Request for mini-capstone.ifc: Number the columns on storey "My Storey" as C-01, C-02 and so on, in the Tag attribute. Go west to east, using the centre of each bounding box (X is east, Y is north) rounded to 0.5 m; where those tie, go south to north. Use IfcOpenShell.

First a look at what the model holds.

```python
import ifcopenshell
import ifcopenshell.util.element
import ifcopenshell.util.placement

model = ifcopenshell.open("mini-capstone.ifc")
print(model.schema)
storey = next(s for s in model.by_type("IfcBuildingStorey") if s.Name == "My Storey")
columns = [e for e in ifcopenshell.util.element.get_decomposition(storey) if e.is_a("IfcColumn")]
for e in sorted(columns, key=lambda e: e.id()):
    origin = ifcopenshell.util.placement.get_local_placement(e.ObjectPlacement)[:3, 3]
    print(e.id(), e.Tag, e.Name, origin.round(2) + 0.0, sep=" | ")
```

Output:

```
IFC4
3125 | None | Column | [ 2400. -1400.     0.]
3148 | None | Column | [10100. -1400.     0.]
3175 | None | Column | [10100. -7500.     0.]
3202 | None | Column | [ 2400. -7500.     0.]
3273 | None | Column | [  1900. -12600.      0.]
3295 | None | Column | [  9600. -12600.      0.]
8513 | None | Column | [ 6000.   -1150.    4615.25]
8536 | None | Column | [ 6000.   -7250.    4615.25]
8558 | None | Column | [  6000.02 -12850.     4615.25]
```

```python
import ifcopenshell
import ifcopenshell.geom
import ifcopenshell.util.element
import ifcopenshell.util.shape

model = ifcopenshell.open("mini-capstone.ifc")
settings = ifcopenshell.geom.settings()
settings.set("use-world-coords", True)


def centre(element):
    shape = ifcopenshell.geom.create_shape(settings, element)
    return ifcopenshell.util.shape.get_bbox_centroid(shape.geometry)


storey = next(s for s in model.by_type("IfcBuildingStorey") if s.Name == "My Storey")
columns = [e for e in ifcopenshell.util.element.get_decomposition(storey) if e.is_a("IfcColumn")]

# Insertion points can sit at a corner or the storey origin, so sort by the geometry (in metres).
centres = {e: centre(e) for e in columns}
columns.sort(key=lambda e: (round(centres[e][0] / 0.5), centres[e][1]))

for i, e in enumerate(columns, start=1):
    number = f"C-{i:02d}"
    e.Tag = number
    print(e.id(), number)

model.write("mini-capstone-out.ifc")
```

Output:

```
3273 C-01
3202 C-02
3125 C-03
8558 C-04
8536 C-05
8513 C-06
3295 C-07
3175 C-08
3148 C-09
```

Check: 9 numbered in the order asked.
